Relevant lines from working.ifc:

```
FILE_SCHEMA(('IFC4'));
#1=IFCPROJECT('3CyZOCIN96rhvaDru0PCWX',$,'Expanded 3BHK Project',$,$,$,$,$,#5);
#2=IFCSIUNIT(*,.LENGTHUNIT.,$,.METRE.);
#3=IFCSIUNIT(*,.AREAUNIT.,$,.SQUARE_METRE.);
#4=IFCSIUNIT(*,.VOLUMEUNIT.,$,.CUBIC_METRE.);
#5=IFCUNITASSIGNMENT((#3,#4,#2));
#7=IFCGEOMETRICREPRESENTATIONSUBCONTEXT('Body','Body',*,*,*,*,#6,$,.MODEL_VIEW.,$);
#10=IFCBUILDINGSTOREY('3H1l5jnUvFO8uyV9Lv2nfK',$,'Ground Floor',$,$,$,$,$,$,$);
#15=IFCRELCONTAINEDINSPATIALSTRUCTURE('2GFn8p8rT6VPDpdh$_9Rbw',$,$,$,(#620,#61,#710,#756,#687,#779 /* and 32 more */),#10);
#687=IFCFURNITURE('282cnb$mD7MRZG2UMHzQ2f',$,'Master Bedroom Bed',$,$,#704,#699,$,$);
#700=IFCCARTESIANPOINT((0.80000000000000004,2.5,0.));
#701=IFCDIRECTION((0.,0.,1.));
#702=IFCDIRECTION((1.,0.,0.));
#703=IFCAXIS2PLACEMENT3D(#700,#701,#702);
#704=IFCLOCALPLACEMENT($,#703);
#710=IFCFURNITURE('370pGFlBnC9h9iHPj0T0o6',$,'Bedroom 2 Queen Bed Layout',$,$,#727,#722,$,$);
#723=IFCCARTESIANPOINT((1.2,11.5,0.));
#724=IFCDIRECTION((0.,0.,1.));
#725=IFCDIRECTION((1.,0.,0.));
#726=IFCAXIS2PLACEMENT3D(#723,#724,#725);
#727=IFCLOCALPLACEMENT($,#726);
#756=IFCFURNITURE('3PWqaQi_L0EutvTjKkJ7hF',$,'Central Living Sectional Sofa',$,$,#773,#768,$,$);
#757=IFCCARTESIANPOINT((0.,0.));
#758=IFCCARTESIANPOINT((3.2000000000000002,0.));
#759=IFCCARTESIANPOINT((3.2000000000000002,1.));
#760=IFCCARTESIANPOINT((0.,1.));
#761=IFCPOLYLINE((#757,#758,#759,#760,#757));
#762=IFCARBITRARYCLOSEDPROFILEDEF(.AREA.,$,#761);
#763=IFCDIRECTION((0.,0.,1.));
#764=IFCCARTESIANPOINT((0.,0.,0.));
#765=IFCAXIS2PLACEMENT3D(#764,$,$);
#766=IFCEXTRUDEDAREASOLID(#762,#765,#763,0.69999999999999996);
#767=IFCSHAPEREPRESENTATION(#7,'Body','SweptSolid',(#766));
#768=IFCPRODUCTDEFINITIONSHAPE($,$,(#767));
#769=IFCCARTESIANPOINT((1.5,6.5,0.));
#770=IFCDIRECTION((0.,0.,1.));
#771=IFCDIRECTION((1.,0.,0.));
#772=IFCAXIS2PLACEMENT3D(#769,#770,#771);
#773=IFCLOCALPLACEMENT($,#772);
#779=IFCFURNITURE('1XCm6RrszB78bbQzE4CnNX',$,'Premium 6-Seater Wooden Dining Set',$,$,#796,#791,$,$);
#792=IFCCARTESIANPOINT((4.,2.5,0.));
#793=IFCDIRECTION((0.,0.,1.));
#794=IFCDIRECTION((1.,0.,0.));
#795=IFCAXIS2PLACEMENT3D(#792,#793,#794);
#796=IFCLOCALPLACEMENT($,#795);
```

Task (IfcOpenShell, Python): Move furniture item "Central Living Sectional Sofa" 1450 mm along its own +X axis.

```python
import ifcopenshell
import ifcopenshell.api.geometry
import ifcopenshell.util.placement
import ifcopenshell.util.unit

model = ifcopenshell.open("working.ifc")
unit_scale = ifcopenshell.util.unit.calculate_unit_scale(model)

item = model.by_id(756)
matrix = ifcopenshell.util.placement.get_local_placement(item.ObjectPlacement)
matrix[:3, 3] += matrix[:3, 0] * 1.45 / unit_scale
ifcopenshell.api.geometry.edit_object_placement(model, product=item, matrix=matrix, is_si=False)

print(ifcopenshell.util.placement.get_local_placement(item.ObjectPlacement).round(3) + 0.0)

model.write("working_v2.ifc")
```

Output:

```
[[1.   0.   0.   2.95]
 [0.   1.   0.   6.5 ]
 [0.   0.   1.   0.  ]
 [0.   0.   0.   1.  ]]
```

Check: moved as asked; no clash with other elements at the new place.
